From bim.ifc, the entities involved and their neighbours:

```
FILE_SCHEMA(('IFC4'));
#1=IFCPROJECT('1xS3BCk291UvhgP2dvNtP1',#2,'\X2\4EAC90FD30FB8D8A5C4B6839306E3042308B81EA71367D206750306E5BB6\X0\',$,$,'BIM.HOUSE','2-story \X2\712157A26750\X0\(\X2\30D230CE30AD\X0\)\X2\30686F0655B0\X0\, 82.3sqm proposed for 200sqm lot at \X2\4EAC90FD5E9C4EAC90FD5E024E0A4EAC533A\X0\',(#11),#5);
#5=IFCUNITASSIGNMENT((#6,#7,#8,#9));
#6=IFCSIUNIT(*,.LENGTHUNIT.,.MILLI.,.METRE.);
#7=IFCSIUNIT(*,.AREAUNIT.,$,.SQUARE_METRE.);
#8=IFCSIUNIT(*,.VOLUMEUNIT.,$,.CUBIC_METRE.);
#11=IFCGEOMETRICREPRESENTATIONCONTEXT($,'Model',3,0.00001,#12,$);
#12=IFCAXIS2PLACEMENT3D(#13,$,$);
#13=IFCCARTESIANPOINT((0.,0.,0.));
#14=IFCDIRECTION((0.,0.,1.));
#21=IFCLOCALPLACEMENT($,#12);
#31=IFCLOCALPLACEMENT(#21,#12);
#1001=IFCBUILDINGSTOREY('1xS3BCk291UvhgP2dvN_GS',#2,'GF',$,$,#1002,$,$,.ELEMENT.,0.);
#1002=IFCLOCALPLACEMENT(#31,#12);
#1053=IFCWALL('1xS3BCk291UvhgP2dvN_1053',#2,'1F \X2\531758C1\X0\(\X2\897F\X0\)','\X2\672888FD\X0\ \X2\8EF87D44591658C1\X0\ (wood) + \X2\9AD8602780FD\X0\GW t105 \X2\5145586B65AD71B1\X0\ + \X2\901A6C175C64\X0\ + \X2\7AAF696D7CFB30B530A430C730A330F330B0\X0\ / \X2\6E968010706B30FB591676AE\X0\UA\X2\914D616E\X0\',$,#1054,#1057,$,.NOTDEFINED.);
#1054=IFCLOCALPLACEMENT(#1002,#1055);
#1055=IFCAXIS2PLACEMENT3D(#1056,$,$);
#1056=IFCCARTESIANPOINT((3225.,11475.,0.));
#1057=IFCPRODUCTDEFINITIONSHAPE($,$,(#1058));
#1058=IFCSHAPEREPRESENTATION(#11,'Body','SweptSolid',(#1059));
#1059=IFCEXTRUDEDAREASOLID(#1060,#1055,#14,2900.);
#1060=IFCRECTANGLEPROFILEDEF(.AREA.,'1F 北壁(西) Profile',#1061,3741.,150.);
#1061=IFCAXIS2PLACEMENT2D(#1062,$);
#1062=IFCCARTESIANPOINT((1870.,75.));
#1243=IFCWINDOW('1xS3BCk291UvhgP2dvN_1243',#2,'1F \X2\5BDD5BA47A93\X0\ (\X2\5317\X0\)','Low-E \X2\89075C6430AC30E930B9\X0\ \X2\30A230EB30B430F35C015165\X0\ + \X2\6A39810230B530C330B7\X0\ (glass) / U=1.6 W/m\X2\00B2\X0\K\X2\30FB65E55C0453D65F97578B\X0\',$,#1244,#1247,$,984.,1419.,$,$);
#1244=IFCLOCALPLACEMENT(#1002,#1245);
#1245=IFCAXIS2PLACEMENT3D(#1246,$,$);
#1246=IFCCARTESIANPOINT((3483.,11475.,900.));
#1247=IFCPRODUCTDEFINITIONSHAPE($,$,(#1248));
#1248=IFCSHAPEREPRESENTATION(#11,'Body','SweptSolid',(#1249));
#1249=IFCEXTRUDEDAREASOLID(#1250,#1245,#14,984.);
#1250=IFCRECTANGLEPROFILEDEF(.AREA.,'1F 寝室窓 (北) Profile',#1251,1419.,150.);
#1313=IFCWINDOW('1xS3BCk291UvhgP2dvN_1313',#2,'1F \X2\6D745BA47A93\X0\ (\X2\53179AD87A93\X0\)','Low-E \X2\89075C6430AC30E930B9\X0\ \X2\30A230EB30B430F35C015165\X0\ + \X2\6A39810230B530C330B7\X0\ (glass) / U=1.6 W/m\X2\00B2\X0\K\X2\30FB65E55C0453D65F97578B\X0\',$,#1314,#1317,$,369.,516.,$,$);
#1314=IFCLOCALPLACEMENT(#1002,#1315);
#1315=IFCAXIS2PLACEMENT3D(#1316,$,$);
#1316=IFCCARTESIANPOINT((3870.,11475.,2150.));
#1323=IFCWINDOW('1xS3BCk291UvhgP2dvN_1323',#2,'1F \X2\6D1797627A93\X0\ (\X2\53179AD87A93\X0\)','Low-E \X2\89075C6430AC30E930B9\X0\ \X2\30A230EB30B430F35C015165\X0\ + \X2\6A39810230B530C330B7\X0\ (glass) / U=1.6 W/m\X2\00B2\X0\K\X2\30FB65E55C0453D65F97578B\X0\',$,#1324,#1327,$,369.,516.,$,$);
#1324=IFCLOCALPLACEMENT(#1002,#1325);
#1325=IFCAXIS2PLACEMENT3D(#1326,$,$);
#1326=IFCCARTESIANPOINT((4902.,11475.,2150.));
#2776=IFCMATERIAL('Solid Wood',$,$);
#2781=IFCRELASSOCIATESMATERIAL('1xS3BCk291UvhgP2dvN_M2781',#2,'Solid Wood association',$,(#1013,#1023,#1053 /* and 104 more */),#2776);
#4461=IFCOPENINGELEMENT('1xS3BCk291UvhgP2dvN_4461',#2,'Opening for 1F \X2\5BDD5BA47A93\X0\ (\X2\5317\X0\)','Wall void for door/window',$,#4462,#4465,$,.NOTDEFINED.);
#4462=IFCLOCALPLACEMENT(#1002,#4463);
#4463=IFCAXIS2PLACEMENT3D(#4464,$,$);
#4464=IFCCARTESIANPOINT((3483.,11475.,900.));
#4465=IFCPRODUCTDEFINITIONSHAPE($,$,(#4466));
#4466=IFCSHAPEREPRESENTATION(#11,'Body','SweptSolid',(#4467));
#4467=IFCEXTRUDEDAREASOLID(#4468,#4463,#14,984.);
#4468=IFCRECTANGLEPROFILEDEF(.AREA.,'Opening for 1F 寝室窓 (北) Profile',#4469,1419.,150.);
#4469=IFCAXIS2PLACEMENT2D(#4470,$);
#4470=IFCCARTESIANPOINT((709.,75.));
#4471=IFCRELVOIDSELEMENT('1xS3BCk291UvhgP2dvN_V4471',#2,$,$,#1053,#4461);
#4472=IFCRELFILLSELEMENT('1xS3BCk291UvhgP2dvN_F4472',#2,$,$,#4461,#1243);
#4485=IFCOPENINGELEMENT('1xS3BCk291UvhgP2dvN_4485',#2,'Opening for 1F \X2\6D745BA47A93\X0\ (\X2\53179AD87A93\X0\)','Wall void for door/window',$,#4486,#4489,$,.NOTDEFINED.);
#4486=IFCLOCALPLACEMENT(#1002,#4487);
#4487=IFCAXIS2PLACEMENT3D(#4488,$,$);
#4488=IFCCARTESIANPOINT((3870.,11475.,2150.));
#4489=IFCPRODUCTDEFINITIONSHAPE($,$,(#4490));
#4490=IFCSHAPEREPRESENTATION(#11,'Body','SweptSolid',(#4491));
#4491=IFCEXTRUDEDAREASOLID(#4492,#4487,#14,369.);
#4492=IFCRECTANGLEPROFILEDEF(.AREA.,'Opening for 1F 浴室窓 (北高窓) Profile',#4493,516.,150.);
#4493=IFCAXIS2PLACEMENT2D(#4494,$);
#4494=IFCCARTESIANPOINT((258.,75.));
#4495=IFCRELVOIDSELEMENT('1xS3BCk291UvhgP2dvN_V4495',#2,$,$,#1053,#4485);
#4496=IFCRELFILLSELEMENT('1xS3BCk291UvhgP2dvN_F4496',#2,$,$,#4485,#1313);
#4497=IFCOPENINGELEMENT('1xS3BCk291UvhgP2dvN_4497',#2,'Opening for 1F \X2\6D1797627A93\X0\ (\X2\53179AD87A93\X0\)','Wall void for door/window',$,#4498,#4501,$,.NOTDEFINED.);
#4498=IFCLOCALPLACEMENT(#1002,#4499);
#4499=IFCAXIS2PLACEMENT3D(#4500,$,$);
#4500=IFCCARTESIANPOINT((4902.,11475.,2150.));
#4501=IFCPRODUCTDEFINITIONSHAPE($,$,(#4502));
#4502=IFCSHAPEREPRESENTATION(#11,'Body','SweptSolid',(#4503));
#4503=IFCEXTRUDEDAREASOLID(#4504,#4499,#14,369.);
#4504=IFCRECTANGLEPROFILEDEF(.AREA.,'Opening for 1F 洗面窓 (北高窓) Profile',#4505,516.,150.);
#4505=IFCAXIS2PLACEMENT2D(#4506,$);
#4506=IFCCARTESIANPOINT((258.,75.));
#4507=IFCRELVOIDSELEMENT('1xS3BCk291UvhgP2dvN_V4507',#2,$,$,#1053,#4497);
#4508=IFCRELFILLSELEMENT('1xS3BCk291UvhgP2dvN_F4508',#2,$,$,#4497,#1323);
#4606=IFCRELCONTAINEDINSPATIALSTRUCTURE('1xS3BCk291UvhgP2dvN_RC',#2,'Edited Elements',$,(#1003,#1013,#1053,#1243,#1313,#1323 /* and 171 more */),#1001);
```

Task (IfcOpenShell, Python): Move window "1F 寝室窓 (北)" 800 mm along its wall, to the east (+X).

```python
import ifcopenshell
import ifcopenshell.api.geometry
import ifcopenshell.util.placement
import ifcopenshell.util.unit

model = ifcopenshell.open("bim.ifc")
unit_scale = ifcopenshell.util.unit.calculate_unit_scale(model)

window = model.by_guid("1xS3BCk291UvhgP2dvN_1243")
opening = window.FillsVoids[0].RelatingOpeningElement
wall = opening.VoidsElements[0].RelatingBuildingElement

wall_matrix = ifcopenshell.util.placement.get_local_placement(wall.ObjectPlacement)
shift = wall_matrix[:3, 0] * 0.8 / unit_scale
before = ifcopenshell.util.placement.get_local_placement(window.ObjectPlacement)[:3, 3].copy()

# The window is not placed relative to its opening, so move both.
for product in (opening, window):
    matrix = ifcopenshell.util.placement.get_local_placement(product.ObjectPlacement)
    matrix[:3, 3] += shift
    ifcopenshell.api.geometry.edit_object_placement(model, product=product, matrix=matrix, is_si=False)

after = ifcopenshell.util.placement.get_local_placement(window.ObjectPlacement)[:3, 3]
print("window moved by", (after - before).round(3) + 0.0)

model.write("bim_edited.ifc")
```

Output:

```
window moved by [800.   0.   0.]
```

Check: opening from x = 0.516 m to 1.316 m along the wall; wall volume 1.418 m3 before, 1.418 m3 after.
